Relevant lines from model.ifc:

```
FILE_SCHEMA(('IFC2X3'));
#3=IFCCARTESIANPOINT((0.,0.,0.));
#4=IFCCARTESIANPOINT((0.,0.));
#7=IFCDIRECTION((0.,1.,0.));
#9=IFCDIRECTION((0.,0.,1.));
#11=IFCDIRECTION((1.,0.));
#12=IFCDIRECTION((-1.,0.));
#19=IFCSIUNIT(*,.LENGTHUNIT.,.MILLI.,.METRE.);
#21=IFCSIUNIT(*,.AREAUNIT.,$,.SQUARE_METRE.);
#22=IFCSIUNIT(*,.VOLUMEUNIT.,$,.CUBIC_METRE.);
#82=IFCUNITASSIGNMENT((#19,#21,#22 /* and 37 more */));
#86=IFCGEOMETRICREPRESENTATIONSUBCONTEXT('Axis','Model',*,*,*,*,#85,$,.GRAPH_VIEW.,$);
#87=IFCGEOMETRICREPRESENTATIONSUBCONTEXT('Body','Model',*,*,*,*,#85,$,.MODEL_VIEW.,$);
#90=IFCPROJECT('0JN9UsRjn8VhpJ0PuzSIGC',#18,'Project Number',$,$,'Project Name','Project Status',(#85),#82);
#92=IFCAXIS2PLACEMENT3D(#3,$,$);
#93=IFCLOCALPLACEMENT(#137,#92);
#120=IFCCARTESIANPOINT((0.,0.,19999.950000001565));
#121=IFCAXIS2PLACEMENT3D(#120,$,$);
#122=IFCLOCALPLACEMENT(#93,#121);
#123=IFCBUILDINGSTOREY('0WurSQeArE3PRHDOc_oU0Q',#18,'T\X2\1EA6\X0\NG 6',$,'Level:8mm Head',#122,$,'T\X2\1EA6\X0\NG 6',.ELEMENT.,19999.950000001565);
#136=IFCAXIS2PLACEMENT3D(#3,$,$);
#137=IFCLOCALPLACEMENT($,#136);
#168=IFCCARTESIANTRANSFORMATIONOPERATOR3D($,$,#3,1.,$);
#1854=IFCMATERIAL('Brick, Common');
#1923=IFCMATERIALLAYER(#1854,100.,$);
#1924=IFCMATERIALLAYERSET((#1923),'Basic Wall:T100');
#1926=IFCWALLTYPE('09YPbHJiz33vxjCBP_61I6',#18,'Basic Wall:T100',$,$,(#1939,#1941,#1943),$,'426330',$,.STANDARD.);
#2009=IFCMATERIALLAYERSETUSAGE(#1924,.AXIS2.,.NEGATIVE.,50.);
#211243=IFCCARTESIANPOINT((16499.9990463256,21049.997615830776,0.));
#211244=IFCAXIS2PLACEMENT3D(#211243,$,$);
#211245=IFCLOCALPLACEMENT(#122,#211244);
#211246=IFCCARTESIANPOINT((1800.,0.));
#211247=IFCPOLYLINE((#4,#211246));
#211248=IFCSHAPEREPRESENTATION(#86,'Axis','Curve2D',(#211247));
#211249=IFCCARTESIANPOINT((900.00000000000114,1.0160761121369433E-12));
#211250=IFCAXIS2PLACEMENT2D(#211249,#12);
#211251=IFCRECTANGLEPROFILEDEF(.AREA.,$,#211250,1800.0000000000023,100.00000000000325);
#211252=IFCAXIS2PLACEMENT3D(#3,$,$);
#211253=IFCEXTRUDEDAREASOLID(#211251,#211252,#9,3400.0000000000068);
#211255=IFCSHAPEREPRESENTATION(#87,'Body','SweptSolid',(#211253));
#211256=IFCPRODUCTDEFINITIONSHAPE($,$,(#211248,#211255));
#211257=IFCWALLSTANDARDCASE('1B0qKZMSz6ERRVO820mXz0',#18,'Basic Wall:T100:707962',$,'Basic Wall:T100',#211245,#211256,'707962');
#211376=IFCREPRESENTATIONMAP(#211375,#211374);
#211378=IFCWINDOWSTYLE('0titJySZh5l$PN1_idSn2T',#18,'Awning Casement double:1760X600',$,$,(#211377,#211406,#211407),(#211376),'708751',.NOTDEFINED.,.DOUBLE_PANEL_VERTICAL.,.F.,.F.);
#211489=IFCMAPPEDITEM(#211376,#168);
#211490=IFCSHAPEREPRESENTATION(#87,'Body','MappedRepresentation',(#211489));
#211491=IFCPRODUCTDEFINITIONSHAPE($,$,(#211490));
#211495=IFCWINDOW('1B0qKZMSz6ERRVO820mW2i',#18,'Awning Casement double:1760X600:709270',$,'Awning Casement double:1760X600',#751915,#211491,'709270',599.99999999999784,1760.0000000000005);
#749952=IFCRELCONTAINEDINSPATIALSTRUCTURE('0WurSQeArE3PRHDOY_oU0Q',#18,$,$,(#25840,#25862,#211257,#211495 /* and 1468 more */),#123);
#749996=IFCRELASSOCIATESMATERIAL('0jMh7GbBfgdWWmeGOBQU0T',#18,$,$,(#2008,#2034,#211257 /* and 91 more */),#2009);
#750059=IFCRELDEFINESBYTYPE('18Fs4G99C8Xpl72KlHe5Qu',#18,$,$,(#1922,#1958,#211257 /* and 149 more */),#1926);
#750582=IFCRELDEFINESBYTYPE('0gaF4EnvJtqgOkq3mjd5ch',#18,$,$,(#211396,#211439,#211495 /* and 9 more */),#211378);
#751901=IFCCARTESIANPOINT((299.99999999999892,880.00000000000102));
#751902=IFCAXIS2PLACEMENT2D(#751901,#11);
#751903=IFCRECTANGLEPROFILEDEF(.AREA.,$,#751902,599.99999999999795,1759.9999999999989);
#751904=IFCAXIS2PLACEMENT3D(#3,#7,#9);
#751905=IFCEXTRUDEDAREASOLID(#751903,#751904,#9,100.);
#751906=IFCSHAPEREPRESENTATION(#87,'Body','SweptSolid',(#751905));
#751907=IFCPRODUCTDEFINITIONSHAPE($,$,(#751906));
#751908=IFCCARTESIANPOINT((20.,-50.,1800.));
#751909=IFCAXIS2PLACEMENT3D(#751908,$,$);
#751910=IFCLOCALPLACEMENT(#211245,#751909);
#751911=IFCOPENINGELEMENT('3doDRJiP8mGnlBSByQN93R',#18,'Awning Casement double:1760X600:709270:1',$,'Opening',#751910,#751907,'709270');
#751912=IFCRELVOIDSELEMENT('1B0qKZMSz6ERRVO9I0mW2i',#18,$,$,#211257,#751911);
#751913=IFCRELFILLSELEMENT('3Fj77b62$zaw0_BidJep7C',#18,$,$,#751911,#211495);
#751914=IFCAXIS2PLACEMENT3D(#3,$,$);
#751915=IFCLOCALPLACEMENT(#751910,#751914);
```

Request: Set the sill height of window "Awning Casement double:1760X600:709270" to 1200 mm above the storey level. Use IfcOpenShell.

```python
import numpy as np
import ifcopenshell
import ifcopenshell.api.geometry
import ifcopenshell.geom
import ifcopenshell.util.element
import ifcopenshell.util.placement
import ifcopenshell.util.shape
import ifcopenshell.util.unit

model = ifcopenshell.open("model.ifc")
unit_scale = ifcopenshell.util.unit.calculate_unit_scale(model)

window = model.by_id(211495)
opening = window.FillsVoids[0].RelatingOpeningElement
storey = ifcopenshell.util.element.get_container(window, ifc_class="IfcBuildingStorey")
level = ifcopenshell.util.placement.get_local_placement(storey.ObjectPlacement)[2, 3]

# The opening's origin need not be at the sill, so measure its lowest point.
shape = ifcopenshell.geom.create_shape(ifcopenshell.geom.settings(), opening)
bottom = ifcopenshell.util.shape.get_shape_bottom_elevation(shape, shape.geometry) / unit_scale
dz = level + 1.2 / unit_scale - bottom

shift = np.array([0.0, 0.0, dz])
# The window is placed relative to its opening, so it follows when the opening moves.
matrix = ifcopenshell.util.placement.get_local_placement(opening.ObjectPlacement)
matrix[:3, 3] += shift
ifcopenshell.api.geometry.edit_object_placement(
    model, product=opening, matrix=matrix, is_si=False, should_transform_children=True
)

print(f"moved by {dz * unit_scale:+.3f} m")

model.write("model_v2.ifc")
```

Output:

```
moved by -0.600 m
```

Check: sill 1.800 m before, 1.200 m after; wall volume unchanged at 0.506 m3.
